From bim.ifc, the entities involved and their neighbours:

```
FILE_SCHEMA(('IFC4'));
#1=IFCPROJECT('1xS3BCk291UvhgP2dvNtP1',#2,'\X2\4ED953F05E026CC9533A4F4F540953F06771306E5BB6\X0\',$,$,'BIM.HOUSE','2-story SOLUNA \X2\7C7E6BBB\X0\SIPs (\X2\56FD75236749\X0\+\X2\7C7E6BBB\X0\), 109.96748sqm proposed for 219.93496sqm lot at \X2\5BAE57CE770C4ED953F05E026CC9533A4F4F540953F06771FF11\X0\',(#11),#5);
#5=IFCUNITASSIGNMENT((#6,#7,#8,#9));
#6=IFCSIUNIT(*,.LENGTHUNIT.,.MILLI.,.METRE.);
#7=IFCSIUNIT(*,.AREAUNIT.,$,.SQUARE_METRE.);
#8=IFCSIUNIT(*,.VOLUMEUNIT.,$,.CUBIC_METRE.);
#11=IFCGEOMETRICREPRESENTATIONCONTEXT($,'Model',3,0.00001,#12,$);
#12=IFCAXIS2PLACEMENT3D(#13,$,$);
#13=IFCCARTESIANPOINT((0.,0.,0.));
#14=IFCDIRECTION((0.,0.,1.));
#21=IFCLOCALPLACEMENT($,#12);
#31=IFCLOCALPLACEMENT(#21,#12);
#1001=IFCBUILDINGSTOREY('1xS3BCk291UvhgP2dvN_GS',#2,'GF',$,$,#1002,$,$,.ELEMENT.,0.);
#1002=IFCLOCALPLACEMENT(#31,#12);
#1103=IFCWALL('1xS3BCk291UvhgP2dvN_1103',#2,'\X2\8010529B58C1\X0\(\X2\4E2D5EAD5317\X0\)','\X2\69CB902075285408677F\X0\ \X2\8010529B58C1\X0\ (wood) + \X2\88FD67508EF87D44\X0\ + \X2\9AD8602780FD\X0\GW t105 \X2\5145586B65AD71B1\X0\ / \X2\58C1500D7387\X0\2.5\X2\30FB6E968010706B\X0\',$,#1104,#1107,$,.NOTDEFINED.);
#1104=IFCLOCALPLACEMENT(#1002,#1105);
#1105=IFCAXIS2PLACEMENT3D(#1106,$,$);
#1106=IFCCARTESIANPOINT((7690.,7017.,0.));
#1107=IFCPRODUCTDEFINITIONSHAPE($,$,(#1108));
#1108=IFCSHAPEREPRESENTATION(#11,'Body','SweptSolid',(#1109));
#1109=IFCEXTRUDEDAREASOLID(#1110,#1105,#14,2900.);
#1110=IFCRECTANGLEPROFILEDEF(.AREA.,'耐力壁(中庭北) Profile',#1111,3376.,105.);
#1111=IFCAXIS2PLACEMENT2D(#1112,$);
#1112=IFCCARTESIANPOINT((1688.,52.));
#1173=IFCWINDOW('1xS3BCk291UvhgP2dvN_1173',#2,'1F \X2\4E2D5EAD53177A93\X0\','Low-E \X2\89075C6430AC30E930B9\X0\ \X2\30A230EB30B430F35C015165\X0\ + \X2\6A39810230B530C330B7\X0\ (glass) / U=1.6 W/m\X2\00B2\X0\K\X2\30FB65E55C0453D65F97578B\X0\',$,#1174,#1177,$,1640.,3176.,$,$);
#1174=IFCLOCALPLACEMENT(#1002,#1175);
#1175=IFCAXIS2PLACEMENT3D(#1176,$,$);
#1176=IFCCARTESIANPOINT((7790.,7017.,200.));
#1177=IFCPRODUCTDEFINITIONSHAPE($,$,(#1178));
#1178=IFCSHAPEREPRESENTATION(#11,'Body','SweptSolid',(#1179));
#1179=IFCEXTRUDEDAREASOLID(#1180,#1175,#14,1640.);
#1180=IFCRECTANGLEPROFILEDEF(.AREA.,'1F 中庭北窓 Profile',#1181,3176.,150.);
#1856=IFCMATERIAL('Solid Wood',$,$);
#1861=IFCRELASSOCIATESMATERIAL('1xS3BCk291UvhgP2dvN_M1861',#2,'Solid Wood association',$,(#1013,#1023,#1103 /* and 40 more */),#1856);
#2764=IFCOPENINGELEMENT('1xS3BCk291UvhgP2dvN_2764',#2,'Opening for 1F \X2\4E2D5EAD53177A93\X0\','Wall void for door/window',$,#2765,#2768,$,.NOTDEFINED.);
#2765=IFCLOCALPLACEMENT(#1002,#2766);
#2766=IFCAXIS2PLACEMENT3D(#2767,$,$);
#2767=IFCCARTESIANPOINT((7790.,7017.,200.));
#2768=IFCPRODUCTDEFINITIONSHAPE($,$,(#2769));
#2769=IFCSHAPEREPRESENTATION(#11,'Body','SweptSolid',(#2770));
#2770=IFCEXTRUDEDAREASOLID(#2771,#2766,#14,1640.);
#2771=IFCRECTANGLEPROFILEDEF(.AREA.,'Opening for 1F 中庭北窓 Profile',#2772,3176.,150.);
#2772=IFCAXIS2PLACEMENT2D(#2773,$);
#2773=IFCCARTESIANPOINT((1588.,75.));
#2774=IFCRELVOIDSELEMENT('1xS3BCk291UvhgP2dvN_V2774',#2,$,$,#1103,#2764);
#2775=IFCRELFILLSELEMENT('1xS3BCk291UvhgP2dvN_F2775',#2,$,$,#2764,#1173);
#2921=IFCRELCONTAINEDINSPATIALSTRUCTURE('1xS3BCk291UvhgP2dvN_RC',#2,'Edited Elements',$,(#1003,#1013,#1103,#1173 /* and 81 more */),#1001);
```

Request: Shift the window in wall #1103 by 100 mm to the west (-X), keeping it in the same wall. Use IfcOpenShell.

```python
import ifcopenshell
import ifcopenshell.api.geometry
import ifcopenshell.util.placement

model = ifcopenshell.open("bim.ifc")

window = model.by_guid("1xS3BCk291UvhgP2dvN_1173")
opening = window.FillsVoids[0].RelatingOpeningElement
wall = opening.VoidsElements[0].RelatingBuildingElement

wall_matrix = ifcopenshell.util.placement.get_local_placement(wall.ObjectPlacement)
shift = wall_matrix[:3, 0] * -100.0
before = ifcopenshell.util.placement.get_local_placement(window.ObjectPlacement)[:3, 3].copy()

# The window is not placed relative to its opening, so move both.
for product in (opening, window):
    matrix = ifcopenshell.util.placement.get_local_placement(product.ObjectPlacement)
    matrix[:3, 3] += shift
    ifcopenshell.api.geometry.edit_object_placement(model, product=product, matrix=matrix, is_si=False)

after = ifcopenshell.util.placement.get_local_placement(window.ObjectPlacement)[:3, 3]
print("window moved by", (after - before).round(3) + 0.0)

model.write("bim_v2.ifc")
```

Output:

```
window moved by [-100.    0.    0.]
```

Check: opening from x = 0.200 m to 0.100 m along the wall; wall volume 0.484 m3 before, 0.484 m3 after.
